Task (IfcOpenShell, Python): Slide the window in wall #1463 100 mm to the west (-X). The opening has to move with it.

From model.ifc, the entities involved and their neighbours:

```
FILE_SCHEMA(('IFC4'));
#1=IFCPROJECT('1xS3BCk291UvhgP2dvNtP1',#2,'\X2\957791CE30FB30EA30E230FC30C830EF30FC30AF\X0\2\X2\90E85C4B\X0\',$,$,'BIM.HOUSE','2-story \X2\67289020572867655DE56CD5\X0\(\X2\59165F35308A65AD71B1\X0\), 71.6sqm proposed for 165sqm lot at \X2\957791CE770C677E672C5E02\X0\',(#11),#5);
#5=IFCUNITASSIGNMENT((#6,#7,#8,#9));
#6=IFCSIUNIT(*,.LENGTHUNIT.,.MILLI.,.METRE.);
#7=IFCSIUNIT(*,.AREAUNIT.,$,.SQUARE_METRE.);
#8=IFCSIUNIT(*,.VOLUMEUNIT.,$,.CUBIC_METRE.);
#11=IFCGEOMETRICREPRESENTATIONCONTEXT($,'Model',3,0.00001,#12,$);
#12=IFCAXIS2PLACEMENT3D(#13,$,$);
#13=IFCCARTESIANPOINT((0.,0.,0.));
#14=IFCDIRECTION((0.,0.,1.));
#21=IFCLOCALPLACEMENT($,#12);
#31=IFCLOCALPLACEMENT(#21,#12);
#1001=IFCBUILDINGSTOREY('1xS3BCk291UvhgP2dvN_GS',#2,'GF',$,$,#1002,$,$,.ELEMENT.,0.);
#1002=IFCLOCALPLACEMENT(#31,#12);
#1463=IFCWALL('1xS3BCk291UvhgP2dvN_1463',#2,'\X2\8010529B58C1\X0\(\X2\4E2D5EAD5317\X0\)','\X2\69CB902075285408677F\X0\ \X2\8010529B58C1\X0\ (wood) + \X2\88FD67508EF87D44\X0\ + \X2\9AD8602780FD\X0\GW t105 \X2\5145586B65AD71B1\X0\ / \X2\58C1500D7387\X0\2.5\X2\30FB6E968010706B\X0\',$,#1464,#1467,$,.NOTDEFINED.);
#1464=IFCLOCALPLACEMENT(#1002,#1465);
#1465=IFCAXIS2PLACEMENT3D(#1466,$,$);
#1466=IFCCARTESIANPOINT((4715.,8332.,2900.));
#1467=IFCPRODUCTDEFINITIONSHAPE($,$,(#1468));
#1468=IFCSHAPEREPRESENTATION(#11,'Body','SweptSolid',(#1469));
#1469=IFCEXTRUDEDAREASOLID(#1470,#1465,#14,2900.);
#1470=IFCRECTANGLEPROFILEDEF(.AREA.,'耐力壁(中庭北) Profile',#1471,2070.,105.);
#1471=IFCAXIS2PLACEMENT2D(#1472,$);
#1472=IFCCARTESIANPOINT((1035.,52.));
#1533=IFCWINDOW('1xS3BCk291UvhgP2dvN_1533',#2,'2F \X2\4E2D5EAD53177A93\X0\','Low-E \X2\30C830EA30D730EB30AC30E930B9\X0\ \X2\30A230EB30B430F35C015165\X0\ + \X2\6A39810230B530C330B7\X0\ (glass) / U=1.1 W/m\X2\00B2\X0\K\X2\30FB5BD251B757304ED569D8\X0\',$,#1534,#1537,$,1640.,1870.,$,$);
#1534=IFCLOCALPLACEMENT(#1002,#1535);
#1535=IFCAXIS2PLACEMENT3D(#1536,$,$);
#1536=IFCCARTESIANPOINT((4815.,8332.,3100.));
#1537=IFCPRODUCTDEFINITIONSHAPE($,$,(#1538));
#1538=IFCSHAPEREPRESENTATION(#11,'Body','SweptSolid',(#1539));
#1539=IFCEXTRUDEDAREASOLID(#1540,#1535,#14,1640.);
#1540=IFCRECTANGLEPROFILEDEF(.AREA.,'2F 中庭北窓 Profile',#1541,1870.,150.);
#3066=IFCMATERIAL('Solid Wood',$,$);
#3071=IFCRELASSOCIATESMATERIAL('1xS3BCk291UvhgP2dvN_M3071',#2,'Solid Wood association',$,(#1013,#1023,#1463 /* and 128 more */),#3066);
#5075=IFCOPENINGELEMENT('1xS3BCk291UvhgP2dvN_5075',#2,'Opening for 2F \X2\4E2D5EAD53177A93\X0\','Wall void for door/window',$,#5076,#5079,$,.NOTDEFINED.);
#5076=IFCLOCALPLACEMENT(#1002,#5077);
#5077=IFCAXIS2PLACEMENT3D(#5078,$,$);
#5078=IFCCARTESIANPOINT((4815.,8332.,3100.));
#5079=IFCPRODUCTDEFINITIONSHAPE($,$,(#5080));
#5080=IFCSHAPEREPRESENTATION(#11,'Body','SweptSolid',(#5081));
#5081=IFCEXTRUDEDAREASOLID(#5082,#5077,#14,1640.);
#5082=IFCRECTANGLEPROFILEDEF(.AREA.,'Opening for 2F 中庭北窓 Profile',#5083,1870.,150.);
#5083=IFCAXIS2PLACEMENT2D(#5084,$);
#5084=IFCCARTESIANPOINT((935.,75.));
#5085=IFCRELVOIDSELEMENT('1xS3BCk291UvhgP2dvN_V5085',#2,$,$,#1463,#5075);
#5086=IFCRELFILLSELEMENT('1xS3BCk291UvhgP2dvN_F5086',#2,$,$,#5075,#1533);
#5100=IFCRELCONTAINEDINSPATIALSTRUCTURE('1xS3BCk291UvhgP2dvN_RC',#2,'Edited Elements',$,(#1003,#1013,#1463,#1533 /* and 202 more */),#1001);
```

```python
import ifcopenshell
import ifcopenshell.api.geometry
import ifcopenshell.util.placement

model = ifcopenshell.open("model.ifc")

window = model.by_id(1533)
opening = window.FillsVoids[0].RelatingOpeningElement
wall = opening.VoidsElements[0].RelatingBuildingElement

wall_matrix = ifcopenshell.util.placement.get_local_placement(wall.ObjectPlacement)
shift = wall_matrix[:3, 0] * -100.0
before = ifcopenshell.util.placement.get_local_placement(window.ObjectPlacement)[:3, 3].copy()

# The window is not placed relative to its opening, so move both.
for product in (opening, window):
    matrix = ifcopenshell.util.placement.get_local_placement(product.ObjectPlacement)
    matrix[:3, 3] += shift
    ifcopenshell.api.geometry.edit_object_placement(model, product=product, matrix=matrix, is_si=False)

after = ifcopenshell.util.placement.get_local_placement(window.ObjectPlacement)[:3, 3]
print("window moved by", (after - before).round(3) + 0.0)

model.write("model-out.ifc")
```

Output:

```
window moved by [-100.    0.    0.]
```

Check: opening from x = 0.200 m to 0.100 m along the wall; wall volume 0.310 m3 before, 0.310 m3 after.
